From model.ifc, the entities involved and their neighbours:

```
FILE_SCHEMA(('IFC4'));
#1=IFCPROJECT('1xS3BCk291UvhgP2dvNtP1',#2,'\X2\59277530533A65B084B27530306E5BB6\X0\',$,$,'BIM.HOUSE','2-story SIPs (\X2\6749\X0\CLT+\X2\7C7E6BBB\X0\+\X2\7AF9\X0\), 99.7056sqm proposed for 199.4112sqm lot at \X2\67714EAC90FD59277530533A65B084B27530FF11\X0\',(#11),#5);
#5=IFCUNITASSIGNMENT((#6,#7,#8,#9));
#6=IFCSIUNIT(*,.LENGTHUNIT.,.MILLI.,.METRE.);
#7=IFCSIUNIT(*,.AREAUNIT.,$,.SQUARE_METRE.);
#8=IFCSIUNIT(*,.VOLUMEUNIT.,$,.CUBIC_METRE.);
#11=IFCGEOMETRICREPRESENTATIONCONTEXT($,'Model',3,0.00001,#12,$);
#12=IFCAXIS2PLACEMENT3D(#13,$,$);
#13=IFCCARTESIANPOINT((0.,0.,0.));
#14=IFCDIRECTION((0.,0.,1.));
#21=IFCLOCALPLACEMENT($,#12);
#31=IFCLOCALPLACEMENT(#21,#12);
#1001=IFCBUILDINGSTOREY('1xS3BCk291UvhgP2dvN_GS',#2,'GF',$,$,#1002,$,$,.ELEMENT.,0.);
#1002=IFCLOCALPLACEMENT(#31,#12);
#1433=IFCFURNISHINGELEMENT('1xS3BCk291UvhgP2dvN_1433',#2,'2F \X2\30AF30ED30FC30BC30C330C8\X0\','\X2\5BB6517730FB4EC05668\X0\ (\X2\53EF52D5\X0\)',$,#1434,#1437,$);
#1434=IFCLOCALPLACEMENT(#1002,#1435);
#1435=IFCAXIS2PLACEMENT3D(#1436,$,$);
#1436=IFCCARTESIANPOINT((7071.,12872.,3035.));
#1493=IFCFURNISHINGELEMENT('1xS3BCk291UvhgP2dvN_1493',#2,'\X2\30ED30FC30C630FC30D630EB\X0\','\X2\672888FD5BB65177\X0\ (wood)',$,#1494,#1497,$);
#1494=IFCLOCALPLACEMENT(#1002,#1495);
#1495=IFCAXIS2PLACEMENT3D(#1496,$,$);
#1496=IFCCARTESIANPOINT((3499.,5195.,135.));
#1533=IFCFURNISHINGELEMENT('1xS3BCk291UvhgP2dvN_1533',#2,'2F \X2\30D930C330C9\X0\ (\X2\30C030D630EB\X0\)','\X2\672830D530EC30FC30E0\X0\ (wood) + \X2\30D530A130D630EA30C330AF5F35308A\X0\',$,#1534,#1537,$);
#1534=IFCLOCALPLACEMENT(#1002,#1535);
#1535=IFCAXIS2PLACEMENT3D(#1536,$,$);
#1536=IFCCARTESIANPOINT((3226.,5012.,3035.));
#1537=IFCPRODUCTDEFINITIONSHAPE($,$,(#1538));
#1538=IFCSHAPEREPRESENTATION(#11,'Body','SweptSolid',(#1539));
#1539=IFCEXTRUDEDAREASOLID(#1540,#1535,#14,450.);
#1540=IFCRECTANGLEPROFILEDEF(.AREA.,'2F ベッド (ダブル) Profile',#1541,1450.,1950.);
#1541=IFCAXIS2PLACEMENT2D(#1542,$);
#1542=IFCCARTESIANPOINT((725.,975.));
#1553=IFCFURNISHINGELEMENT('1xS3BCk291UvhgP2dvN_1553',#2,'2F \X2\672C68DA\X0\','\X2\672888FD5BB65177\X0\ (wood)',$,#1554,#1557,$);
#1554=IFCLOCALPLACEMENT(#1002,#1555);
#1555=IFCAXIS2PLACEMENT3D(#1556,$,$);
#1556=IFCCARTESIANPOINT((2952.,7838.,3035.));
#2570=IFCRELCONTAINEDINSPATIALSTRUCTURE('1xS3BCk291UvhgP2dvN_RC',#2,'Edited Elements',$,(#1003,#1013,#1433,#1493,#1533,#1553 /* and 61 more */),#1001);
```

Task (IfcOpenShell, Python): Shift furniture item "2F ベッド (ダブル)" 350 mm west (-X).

```python
import ifcopenshell
import ifcopenshell.api.geometry
import ifcopenshell.util.placement

model = ifcopenshell.open("model.ifc")

item = model.by_id(1533)
matrix = ifcopenshell.util.placement.get_local_placement(item.ObjectPlacement)
matrix[0, 3] -= 350.0
ifcopenshell.api.geometry.edit_object_placement(model, product=item, matrix=matrix, is_si=False)

print(ifcopenshell.util.placement.get_local_placement(item.ObjectPlacement).round(3) + 0.0)

model.write("model_edited.ifc")
```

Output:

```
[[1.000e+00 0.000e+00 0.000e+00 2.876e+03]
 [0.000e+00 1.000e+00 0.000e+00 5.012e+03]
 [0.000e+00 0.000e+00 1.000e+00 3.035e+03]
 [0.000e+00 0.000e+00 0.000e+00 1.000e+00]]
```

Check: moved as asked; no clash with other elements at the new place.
